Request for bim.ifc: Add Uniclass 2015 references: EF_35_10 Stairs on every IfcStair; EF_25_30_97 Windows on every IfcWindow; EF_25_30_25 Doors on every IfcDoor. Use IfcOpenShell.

First a look at what the model holds.

```python
import ifcopenshell

model = ifcopenshell.open("bim.ifc")
print(model.schema)
print("classifications:", [c.Name for c in model.by_type("IfcClassification")])
for ifc_class in ("IfcDoor", "IfcRoof", "IfcStair", "IfcWall", "IfcWindow"):
    print(ifc_class, len(model.by_type(ifc_class)))
```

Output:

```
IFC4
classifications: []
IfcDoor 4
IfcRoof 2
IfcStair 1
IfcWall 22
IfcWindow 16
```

```python
import ifcopenshell
import ifcopenshell.api.classification

model = ifcopenshell.open("bim.ifc")

system = ifcopenshell.api.classification.add_classification(model, classification="Uniclass 2015")

codes = {
    "IfcStair": ("EF_35_10", "Stairs"),
    "IfcWindow": ("EF_25_30_97", "Windows"),
    "IfcDoor": ("EF_25_30_25", "Doors"),
}
for ifc_class, (code, name) in codes.items():
    products = model.by_type(ifc_class)
    ifcopenshell.api.classification.add_reference(
        model, products=products, classification=system, identification=code, name=name
    )
    print(code, len(products))

model.write("bim_edited.ifc")
```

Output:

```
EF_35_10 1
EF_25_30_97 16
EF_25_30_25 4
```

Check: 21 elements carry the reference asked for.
